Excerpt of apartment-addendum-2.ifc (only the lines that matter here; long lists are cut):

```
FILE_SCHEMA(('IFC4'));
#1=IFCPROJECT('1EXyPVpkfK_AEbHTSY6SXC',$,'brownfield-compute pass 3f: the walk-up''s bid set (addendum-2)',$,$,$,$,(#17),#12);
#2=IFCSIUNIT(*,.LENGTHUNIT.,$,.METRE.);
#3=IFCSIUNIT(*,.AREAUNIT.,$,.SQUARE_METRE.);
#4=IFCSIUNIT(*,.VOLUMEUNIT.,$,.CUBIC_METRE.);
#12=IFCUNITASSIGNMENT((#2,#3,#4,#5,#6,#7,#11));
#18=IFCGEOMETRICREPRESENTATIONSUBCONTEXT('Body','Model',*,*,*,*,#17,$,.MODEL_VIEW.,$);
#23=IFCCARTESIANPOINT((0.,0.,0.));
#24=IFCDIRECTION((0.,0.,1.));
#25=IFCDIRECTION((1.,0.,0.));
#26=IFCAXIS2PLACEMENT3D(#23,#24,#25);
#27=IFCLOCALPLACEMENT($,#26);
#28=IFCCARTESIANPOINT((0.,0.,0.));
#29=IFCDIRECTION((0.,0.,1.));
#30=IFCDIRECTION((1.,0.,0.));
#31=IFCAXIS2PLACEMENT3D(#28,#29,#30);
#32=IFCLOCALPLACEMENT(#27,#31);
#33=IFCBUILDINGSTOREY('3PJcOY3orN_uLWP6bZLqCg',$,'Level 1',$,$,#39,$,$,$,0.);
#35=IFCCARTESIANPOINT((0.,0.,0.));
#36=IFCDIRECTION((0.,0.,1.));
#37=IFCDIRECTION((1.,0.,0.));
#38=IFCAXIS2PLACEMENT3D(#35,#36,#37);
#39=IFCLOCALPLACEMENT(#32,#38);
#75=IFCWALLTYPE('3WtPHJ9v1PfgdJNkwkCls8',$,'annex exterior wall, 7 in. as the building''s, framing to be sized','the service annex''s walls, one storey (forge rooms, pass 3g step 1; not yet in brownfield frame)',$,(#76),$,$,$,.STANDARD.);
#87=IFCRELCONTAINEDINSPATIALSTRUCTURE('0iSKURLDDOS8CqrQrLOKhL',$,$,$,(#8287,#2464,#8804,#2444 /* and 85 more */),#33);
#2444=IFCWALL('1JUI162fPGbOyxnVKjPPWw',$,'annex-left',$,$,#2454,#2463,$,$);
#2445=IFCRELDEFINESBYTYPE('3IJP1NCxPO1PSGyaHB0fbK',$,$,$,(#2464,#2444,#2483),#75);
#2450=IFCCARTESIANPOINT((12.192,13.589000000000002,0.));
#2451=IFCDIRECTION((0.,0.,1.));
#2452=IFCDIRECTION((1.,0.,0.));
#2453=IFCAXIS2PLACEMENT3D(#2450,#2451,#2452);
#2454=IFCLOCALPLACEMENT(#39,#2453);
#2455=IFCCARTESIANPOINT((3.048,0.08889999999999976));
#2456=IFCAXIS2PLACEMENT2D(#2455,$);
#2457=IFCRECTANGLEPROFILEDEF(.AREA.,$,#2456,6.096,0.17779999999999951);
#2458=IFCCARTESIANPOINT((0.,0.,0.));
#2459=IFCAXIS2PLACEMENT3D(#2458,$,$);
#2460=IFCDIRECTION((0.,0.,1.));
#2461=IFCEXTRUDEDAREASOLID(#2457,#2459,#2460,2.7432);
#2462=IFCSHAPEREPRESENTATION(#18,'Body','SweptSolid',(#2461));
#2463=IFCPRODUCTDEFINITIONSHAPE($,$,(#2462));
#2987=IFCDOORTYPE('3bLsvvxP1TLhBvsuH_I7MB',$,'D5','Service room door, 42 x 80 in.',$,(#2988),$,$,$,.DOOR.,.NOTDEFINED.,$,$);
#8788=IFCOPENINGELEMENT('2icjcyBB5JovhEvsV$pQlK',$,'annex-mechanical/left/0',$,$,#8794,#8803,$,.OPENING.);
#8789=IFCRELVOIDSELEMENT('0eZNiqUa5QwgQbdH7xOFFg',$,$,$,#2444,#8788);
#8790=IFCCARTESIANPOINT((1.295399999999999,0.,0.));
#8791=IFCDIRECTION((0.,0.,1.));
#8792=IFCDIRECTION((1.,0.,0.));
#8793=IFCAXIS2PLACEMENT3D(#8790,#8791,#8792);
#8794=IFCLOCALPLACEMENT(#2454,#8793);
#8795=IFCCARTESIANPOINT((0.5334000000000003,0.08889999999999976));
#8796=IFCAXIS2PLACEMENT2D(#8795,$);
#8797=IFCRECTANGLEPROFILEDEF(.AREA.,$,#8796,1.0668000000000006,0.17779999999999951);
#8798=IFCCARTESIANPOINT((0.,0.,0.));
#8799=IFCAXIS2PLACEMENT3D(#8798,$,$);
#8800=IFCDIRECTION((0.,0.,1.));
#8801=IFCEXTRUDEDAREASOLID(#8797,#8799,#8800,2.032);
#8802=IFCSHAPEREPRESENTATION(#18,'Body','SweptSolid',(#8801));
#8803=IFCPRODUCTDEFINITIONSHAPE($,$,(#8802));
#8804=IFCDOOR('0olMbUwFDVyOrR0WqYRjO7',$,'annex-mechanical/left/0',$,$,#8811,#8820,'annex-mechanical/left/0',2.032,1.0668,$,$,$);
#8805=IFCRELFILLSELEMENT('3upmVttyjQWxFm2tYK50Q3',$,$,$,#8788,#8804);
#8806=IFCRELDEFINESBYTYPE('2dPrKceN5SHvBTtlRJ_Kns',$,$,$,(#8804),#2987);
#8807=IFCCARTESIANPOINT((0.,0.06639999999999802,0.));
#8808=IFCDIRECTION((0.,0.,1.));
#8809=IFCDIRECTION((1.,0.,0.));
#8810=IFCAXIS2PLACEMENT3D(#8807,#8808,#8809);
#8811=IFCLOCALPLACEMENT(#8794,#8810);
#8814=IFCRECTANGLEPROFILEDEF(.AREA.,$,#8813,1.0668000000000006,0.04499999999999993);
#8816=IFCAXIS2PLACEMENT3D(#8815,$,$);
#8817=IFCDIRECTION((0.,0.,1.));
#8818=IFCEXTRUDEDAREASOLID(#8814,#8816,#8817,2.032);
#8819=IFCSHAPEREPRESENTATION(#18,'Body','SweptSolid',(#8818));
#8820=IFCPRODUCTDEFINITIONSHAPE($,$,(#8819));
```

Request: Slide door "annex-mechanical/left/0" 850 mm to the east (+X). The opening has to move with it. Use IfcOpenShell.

```python
import ifcopenshell
import ifcopenshell.api.geometry
import ifcopenshell.util.placement

model = ifcopenshell.open("apartment-addendum-2.ifc")

door = model.by_guid("0olMbUwFDVyOrR0WqYRjO7")
opening = door.FillsVoids[0].RelatingOpeningElement
wall = opening.VoidsElements[0].RelatingBuildingElement

wall_matrix = ifcopenshell.util.placement.get_local_placement(wall.ObjectPlacement)
shift = wall_matrix[:3, 0] * 0.85
before = ifcopenshell.util.placement.get_local_placement(door.ObjectPlacement)[:3, 3].copy()

# The door is placed relative to its opening, so it follows when the opening moves.
matrix = ifcopenshell.util.placement.get_local_placement(opening.ObjectPlacement)
matrix[:3, 3] += shift
ifcopenshell.api.geometry.edit_object_placement(
    model, product=opening, matrix=matrix, is_si=False, should_transform_children=True
)

after = ifcopenshell.util.placement.get_local_placement(door.ObjectPlacement)[:3, 3]
print("door moved by", (after - before).round(3) + 0.0)

model.write("apartment-addendum-2_edited.ifc")
```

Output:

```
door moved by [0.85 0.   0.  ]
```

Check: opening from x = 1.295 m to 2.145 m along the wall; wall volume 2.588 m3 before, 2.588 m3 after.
